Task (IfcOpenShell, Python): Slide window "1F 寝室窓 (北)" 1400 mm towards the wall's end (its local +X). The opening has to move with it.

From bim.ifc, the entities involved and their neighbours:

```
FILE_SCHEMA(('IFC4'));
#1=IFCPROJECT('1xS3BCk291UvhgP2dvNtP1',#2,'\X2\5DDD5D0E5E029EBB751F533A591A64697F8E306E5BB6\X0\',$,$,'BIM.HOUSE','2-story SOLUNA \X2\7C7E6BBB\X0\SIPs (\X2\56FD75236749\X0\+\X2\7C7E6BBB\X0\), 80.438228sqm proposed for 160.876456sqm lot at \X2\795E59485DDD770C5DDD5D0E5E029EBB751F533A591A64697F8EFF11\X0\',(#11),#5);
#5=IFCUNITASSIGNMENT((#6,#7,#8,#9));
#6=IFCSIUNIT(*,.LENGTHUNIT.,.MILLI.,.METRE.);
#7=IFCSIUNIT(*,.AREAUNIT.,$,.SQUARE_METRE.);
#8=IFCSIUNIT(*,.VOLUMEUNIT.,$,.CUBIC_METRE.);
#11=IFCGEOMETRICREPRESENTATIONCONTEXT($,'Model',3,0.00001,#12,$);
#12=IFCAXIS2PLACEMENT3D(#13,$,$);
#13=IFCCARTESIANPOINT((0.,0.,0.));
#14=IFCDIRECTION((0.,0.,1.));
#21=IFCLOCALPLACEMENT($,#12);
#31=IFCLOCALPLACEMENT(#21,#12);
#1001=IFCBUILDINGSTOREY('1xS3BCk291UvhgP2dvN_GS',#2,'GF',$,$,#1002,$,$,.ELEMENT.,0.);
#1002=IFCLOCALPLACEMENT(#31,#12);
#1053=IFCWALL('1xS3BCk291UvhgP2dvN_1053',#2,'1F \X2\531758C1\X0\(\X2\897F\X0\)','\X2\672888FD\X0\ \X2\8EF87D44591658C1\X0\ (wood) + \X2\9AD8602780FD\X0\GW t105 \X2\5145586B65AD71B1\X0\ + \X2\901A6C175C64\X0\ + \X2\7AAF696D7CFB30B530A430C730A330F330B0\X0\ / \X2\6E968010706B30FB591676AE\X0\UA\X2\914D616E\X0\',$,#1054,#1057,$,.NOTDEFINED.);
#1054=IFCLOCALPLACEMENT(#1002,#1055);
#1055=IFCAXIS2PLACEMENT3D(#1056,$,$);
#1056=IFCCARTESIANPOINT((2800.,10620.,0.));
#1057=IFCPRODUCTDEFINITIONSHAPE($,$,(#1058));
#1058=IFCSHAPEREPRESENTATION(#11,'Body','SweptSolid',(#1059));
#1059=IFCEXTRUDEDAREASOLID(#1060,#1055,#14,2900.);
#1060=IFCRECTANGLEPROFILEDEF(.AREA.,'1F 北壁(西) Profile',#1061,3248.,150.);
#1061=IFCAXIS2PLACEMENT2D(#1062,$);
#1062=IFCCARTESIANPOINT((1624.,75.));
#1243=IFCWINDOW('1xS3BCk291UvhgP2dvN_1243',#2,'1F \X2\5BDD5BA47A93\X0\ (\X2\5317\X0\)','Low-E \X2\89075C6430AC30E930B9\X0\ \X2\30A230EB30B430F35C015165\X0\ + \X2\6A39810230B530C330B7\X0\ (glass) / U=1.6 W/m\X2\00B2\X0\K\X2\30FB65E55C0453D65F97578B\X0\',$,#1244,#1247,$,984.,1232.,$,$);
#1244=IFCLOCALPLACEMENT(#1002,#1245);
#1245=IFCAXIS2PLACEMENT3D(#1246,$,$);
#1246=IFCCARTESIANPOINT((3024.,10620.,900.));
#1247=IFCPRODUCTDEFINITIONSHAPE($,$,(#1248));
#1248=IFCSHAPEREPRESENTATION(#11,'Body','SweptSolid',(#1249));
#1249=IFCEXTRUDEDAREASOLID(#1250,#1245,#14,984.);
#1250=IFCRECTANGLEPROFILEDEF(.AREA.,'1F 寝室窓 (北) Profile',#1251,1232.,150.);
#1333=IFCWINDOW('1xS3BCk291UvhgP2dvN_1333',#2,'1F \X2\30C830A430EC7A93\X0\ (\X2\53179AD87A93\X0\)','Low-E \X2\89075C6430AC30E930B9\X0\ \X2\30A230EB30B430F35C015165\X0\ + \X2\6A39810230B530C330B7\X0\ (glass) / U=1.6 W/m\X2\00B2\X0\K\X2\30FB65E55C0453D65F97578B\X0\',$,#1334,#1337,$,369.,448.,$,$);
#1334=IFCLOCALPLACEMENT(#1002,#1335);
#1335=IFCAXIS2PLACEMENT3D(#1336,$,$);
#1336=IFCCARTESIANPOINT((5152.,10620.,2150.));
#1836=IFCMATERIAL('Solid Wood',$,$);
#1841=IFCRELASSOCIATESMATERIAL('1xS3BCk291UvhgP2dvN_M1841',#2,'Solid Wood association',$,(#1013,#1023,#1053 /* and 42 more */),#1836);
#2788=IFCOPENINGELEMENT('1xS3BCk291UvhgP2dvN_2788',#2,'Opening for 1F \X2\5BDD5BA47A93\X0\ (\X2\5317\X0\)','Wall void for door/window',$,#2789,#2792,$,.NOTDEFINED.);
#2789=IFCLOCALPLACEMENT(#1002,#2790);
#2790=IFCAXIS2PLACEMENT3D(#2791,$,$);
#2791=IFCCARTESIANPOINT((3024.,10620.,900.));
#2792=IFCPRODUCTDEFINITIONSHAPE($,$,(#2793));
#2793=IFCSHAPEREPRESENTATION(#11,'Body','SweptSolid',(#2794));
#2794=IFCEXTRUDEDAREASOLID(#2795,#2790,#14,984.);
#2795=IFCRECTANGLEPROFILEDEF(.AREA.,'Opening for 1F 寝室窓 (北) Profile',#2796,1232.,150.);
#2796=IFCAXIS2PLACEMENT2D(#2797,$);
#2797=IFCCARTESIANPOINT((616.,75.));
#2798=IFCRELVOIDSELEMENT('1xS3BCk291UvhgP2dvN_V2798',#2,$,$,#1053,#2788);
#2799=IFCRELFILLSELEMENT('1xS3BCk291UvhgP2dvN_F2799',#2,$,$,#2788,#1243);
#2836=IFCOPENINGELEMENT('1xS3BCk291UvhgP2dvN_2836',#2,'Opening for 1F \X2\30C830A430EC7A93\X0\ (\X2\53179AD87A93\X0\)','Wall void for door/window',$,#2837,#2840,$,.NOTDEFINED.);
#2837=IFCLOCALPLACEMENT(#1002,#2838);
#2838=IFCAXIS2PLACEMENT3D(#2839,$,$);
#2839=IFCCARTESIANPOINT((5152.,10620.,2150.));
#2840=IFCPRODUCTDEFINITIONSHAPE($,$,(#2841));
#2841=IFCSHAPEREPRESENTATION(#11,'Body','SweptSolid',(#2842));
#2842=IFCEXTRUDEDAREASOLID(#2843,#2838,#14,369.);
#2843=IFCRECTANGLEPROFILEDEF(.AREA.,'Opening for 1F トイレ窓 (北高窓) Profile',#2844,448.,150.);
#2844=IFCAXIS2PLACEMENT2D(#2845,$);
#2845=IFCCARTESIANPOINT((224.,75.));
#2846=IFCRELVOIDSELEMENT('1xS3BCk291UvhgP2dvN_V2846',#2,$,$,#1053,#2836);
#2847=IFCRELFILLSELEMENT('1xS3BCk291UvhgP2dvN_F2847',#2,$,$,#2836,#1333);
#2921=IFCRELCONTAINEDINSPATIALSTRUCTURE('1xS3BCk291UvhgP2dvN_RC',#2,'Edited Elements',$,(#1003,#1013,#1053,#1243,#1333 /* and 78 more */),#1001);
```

```python
import ifcopenshell
import ifcopenshell.api.geometry
import ifcopenshell.util.placement

model = ifcopenshell.open("bim.ifc")

window = model.by_id(1243)
opening = window.FillsVoids[0].RelatingOpeningElement
wall = opening.VoidsElements[0].RelatingBuildingElement

wall_matrix = ifcopenshell.util.placement.get_local_placement(wall.ObjectPlacement)
shift = wall_matrix[:3, 0] * 1400.0
before = ifcopenshell.util.placement.get_local_placement(window.ObjectPlacement)[:3, 3].copy()

# The window is not placed relative to its opening, so move both.
for product in (opening, window):
    matrix = ifcopenshell.util.placement.get_local_placement(product.ObjectPlacement)
    matrix[:3, 3] += shift
    ifcopenshell.api.geometry.edit_object_placement(model, product=product, matrix=matrix, is_si=False)

after = ifcopenshell.util.placement.get_local_placement(window.ObjectPlacement)[:3, 3]
print("window moved by", (after - before).round(3) + 0.0)

model.write("bim-out.ifc")
```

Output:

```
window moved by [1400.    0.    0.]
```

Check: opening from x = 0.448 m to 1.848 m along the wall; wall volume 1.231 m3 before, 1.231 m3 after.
